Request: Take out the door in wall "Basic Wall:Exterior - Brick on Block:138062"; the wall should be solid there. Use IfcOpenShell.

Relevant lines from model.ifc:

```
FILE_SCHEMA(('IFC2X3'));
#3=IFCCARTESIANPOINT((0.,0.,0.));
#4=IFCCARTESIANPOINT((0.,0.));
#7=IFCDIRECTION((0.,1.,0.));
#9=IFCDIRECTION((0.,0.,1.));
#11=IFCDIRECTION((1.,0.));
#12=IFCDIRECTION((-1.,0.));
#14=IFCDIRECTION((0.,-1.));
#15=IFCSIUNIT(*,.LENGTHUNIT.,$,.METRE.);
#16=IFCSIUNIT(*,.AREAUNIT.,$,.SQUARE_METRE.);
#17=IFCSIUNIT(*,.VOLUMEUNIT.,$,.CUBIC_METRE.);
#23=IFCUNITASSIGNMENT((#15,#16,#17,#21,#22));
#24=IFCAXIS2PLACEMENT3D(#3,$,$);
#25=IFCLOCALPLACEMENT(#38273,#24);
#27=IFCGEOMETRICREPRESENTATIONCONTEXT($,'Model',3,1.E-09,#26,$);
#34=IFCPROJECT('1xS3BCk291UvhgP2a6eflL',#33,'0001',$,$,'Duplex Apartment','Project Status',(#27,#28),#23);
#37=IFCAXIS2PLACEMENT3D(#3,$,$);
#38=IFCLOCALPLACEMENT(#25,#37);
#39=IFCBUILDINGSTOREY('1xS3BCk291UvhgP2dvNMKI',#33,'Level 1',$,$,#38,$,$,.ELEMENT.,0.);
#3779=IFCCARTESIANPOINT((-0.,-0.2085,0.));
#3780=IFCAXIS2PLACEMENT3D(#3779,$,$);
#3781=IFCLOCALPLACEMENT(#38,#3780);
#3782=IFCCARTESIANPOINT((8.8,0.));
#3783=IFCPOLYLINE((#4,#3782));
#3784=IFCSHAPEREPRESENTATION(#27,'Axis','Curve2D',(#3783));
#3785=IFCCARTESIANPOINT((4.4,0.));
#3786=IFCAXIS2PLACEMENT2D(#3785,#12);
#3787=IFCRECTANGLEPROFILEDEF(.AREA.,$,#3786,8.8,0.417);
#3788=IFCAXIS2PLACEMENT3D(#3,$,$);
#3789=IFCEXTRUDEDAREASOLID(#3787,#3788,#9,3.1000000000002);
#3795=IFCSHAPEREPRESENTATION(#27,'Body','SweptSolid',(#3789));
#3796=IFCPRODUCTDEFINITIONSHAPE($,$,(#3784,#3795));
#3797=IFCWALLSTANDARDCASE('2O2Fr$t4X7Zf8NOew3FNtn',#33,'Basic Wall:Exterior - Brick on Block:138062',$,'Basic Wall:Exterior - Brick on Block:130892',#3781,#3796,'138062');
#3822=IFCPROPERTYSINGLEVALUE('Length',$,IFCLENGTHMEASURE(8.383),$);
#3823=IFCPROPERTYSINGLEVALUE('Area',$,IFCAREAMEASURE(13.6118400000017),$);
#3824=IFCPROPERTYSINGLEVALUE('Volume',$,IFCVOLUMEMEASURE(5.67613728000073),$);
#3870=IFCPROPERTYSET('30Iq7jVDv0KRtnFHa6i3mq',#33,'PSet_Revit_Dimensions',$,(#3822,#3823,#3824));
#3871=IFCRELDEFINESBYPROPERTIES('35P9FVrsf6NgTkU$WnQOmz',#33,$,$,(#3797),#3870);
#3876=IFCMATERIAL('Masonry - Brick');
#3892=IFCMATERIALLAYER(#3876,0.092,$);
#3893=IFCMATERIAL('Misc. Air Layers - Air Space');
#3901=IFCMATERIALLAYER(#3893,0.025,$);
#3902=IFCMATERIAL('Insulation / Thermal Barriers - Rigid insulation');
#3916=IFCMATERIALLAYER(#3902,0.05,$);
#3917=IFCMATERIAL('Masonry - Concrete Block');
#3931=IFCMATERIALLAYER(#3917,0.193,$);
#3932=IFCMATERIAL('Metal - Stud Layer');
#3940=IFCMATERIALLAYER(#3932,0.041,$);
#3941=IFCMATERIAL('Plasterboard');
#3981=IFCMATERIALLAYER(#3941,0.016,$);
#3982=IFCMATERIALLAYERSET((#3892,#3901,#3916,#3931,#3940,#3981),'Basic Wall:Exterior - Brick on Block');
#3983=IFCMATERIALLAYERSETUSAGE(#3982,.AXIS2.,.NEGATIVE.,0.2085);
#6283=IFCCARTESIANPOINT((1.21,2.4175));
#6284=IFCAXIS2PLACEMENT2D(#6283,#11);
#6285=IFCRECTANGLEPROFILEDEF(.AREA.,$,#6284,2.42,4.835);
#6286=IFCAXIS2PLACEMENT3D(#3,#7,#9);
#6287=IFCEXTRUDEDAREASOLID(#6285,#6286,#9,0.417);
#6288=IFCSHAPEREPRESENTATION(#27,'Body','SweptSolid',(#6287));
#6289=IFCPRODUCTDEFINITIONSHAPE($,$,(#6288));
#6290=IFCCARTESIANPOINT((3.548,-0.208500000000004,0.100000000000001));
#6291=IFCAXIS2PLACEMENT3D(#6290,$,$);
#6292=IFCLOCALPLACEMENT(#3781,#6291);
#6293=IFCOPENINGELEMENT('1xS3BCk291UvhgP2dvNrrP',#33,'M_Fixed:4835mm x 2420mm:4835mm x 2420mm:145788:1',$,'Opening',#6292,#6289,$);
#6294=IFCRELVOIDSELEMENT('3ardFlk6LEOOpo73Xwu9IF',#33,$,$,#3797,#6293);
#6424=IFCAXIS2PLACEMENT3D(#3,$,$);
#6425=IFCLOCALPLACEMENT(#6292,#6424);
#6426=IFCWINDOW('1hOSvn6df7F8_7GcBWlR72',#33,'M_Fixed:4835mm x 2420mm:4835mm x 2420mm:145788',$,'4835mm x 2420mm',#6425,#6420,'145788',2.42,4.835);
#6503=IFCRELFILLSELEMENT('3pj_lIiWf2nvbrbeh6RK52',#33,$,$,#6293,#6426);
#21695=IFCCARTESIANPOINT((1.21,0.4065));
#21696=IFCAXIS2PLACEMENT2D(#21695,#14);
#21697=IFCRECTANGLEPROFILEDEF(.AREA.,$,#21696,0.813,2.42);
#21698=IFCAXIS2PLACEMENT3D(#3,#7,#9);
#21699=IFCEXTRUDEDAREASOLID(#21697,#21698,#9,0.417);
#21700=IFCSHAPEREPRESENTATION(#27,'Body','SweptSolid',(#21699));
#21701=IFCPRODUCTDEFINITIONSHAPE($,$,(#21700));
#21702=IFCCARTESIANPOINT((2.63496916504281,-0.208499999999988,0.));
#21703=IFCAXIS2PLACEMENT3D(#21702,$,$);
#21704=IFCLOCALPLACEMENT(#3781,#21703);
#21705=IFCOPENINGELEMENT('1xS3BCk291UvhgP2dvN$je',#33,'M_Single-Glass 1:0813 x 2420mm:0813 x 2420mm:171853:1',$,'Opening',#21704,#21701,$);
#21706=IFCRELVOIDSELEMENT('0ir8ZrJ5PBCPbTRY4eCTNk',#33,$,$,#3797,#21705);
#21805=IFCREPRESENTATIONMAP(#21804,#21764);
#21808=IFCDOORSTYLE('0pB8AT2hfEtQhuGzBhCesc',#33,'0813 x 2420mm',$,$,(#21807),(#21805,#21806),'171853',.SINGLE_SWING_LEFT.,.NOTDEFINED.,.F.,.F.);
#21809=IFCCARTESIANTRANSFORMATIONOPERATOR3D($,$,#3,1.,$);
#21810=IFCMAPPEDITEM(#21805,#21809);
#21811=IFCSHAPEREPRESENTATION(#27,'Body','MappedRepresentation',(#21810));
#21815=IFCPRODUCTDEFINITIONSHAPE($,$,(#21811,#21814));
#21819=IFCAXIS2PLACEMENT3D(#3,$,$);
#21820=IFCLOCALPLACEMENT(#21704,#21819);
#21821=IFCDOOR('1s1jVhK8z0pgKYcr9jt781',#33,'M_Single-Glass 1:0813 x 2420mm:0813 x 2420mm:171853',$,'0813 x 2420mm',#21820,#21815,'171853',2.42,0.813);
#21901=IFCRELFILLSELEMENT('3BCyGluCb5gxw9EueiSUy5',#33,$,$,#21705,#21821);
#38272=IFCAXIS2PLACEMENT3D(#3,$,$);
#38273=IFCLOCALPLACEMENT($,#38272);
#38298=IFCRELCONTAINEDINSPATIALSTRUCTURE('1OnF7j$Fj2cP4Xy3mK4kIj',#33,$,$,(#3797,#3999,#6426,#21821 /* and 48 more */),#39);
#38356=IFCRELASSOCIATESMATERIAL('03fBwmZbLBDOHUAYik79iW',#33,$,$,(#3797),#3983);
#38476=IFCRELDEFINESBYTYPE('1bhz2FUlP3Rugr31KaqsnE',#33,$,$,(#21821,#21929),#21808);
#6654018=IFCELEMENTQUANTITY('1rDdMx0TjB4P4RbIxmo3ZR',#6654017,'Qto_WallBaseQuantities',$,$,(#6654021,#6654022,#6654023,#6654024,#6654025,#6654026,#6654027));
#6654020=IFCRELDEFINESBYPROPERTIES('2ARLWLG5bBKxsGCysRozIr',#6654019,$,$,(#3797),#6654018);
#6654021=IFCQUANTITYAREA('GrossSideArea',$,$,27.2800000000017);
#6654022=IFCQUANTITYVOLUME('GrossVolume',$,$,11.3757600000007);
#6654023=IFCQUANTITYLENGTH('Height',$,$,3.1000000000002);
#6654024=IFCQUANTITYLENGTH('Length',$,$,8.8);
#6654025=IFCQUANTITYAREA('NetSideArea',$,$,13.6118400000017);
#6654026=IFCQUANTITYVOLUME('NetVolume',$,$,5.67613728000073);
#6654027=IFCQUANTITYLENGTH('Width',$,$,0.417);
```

```python
import ifcopenshell
import ifcopenshell.api.feature
import ifcopenshell.api.pset
import ifcopenshell.api.root
import ifcopenshell.geom
import ifcopenshell.util.element
import ifcopenshell.util.shape
import ifcopenshell.util.unit

model = ifcopenshell.open("model.ifc")
area_scale = ifcopenshell.util.unit.calculate_unit_scale(model, "AREAUNIT")
volume_scale = ifcopenshell.util.unit.calculate_unit_scale(model, "VOLUMEUNIT")
settings = ifcopenshell.geom.settings()


def volume(element):
    """Net volume in cubic metres, openings subtracted."""
    shape = ifcopenshell.geom.create_shape(settings, element)
    return ifcopenshell.util.shape.get_volume(shape.geometry)


door = model.by_guid("1s1jVhK8z0pgKYcr9jt781")
opening = door.FillsVoids[0].RelatingOpeningElement
wall = opening.VoidsElements[0].RelatingBuildingElement
before = volume(wall)

ifcopenshell.api.root.remove_product(model, product=door)
ifcopenshell.api.feature.remove_feature(model, feature=opening)

after = volume(wall)
thickness = 0.417  # wall thickness in metres

# Update the wall's stored quantities.
pset = model.by_id(ifcopenshell.util.element.get_pset(wall, "PSet_Revit_Dimensions", should_inherit=False)["id"])
ifcopenshell.api.pset.edit_pset(model, pset=pset, properties={
    "Area": model.create_entity("IfcAreaMeasure", after / thickness / area_scale),
    "Volume": model.create_entity("IfcVolumeMeasure", after / volume_scale),
})
qto = model.by_id(ifcopenshell.util.element.get_pset(wall, "Qto_WallBaseQuantities", should_inherit=False)["id"])
ifcopenshell.api.pset.edit_qto(model, qto=qto, properties={
    "NetSideArea": after / thickness / area_scale,
    "NetVolume": after / volume_scale,
})

print(f"wall volume {before:.3f} -> {after:.3f} m3")

model.write("model_v2.ifc")
```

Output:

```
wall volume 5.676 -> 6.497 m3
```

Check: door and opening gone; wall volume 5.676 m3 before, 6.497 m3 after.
